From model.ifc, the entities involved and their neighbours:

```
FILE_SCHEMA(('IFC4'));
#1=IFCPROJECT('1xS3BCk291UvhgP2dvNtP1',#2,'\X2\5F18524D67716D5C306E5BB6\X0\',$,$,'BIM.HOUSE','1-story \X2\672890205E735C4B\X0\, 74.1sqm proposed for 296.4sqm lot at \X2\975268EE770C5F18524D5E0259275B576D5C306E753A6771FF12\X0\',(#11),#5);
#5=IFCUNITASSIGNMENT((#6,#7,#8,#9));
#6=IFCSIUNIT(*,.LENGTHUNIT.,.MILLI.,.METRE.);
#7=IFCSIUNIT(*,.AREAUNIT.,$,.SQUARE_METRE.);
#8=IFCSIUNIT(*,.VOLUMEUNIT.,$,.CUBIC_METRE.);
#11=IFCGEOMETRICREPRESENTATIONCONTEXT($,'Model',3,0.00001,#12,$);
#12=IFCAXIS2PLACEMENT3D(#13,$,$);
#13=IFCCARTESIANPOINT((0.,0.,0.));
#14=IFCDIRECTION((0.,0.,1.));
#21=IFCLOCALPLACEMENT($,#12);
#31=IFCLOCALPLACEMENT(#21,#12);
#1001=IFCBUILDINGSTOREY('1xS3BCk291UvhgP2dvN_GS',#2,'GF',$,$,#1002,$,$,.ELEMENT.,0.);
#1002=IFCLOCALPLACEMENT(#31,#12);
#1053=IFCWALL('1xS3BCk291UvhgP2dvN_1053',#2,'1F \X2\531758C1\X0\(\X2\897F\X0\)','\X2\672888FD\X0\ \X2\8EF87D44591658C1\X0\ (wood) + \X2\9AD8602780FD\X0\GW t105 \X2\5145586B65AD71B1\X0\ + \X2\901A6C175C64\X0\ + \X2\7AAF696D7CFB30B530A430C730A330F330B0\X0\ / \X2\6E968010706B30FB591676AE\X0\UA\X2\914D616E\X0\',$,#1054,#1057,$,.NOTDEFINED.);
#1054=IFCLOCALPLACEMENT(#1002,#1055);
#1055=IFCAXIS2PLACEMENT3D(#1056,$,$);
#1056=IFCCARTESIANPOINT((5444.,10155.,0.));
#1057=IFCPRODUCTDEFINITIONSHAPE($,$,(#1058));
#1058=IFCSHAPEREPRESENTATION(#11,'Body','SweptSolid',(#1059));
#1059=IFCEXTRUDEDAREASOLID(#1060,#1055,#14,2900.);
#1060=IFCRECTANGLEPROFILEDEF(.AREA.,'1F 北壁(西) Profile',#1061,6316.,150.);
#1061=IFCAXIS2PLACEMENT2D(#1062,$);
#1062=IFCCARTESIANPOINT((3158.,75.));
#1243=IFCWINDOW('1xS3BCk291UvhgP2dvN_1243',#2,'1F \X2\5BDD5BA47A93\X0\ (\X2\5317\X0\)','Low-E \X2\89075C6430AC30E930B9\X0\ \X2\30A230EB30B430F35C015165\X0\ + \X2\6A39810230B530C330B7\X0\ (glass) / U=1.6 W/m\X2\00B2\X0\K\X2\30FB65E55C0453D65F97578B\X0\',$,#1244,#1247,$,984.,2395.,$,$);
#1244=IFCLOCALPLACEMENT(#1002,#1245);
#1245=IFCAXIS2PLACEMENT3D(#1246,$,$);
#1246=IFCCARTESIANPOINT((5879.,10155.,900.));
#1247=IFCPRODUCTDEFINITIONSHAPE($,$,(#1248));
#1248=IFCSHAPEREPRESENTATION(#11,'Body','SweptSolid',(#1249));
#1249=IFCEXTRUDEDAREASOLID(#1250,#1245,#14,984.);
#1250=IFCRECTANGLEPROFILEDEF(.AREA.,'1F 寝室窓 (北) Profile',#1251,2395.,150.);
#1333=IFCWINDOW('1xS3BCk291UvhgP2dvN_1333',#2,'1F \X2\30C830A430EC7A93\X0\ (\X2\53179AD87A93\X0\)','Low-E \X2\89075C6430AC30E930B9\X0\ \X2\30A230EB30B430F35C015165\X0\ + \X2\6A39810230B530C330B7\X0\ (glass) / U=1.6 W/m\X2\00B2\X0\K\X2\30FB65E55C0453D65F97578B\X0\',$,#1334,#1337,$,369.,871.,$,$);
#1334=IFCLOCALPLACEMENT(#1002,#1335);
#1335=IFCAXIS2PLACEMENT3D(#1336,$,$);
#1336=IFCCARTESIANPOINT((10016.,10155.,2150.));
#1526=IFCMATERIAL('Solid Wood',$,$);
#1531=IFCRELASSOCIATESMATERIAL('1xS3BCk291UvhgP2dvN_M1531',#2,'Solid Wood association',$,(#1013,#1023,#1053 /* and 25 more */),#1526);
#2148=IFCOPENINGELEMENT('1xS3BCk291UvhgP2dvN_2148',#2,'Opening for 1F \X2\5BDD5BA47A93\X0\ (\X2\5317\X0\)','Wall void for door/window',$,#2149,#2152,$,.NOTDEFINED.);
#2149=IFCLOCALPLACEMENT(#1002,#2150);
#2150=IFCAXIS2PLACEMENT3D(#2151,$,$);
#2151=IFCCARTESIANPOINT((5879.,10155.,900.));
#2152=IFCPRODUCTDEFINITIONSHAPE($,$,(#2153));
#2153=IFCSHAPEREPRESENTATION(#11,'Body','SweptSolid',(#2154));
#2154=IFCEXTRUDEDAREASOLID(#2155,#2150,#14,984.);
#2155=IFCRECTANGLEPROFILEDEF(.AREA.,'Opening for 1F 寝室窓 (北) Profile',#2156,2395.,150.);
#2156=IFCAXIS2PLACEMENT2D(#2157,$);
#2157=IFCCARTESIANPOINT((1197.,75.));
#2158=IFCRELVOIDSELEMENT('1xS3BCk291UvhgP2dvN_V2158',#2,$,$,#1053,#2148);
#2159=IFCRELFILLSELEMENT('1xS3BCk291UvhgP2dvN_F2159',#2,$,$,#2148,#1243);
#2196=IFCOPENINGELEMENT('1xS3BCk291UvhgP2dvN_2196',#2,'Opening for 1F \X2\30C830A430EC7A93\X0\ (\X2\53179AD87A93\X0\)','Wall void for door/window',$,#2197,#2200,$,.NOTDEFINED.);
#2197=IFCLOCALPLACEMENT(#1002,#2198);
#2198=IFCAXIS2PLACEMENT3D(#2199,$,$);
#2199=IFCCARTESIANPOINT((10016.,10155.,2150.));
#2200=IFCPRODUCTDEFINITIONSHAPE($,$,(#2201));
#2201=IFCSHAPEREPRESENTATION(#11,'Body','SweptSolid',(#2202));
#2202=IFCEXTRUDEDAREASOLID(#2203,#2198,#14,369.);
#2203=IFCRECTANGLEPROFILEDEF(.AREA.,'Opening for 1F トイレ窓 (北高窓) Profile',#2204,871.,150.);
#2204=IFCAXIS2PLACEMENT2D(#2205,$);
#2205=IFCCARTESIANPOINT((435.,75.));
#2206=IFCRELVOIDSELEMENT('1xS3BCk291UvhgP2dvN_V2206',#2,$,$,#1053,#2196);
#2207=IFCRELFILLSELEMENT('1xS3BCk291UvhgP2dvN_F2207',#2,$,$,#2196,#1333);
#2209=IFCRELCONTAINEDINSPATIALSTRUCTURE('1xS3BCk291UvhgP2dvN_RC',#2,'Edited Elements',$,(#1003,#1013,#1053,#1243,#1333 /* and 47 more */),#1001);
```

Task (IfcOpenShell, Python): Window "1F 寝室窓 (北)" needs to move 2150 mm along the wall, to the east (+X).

```python
import ifcopenshell
import ifcopenshell.api.geometry
import ifcopenshell.util.placement

model = ifcopenshell.open("model.ifc")

window = model.by_guid("1xS3BCk291UvhgP2dvN_1243")
opening = window.FillsVoids[0].RelatingOpeningElement
wall = opening.VoidsElements[0].RelatingBuildingElement

wall_matrix = ifcopenshell.util.placement.get_local_placement(wall.ObjectPlacement)
shift = wall_matrix[:3, 0] * 2150.0
before = ifcopenshell.util.placement.get_local_placement(window.ObjectPlacement)[:3, 3].copy()

# The window is not placed relative to its opening, so move both.
for product in (opening, window):
    matrix = ifcopenshell.util.placement.get_local_placement(product.ObjectPlacement)
    matrix[:3, 3] += shift
    ifcopenshell.api.geometry.edit_object_placement(model, product=product, matrix=matrix, is_si=False)

after = ifcopenshell.util.placement.get_local_placement(window.ObjectPlacement)[:3, 3]
print("window moved by", (after - before).round(3) + 0.0)

model.write("model_edited.ifc")
```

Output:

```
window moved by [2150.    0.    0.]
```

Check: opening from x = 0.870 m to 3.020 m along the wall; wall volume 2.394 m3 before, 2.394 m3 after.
